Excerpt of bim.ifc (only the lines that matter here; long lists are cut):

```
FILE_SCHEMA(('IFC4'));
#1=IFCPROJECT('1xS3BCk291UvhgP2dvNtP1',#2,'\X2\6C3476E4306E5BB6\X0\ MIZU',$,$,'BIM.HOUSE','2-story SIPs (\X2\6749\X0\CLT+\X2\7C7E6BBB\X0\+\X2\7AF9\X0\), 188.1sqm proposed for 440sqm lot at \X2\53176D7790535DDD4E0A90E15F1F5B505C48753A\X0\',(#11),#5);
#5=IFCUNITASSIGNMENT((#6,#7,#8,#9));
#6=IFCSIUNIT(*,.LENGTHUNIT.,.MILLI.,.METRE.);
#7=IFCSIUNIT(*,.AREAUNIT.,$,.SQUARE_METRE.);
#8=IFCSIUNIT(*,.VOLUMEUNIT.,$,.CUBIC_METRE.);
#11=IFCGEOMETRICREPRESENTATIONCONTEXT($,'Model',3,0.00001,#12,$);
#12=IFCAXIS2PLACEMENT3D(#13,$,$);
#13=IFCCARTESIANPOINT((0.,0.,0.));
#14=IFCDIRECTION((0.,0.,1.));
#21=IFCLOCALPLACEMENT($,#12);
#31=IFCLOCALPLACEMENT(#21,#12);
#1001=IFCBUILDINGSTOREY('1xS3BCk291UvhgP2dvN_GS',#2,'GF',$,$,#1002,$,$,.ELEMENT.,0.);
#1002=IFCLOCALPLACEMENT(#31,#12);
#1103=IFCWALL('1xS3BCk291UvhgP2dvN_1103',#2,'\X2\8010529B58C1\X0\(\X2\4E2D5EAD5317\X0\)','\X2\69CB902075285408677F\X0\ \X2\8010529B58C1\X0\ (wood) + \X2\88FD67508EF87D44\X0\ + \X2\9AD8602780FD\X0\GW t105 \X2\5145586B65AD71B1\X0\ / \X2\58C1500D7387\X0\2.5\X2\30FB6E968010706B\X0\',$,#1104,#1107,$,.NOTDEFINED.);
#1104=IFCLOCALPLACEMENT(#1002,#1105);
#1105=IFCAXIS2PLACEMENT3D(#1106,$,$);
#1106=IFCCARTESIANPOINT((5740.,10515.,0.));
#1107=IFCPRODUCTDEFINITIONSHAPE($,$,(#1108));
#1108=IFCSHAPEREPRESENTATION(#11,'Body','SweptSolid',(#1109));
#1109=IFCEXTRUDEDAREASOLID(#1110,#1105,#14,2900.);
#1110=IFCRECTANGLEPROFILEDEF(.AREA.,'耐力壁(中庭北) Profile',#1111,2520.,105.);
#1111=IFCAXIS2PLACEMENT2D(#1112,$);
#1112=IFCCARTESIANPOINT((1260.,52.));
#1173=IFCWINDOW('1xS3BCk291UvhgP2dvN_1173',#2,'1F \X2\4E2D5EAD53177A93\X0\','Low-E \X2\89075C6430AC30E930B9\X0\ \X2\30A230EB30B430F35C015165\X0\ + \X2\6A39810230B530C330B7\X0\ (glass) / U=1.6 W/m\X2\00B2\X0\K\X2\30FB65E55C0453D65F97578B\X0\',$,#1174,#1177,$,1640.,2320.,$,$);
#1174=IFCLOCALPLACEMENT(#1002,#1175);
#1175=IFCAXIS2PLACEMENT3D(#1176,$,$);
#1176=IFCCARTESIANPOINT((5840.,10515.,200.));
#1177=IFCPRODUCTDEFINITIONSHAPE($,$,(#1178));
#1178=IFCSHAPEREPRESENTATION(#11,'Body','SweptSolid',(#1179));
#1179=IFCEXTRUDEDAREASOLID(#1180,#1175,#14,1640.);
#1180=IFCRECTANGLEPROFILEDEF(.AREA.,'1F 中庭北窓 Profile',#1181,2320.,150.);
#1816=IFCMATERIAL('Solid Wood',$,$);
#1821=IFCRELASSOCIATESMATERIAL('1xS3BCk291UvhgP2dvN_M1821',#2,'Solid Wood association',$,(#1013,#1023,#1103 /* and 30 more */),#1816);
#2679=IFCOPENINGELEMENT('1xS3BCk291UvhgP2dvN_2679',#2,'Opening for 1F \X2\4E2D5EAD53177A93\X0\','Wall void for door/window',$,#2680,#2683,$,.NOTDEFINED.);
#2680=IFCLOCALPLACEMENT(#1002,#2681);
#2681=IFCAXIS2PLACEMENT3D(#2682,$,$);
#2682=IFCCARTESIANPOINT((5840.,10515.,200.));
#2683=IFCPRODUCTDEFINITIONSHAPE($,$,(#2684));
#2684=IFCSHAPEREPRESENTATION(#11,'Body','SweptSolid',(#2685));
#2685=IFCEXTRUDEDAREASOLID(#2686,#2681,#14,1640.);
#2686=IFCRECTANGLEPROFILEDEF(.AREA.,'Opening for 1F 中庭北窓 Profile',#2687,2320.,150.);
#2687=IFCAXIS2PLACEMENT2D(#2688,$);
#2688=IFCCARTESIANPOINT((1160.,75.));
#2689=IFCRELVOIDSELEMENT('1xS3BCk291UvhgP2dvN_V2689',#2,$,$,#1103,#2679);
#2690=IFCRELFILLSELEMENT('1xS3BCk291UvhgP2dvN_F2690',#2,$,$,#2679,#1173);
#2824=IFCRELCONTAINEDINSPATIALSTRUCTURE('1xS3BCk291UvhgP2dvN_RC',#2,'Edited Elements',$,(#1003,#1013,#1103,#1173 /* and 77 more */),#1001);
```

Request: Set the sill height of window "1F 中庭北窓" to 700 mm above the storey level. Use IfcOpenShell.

```python
import numpy as np
import ifcopenshell
import ifcopenshell.api.geometry
import ifcopenshell.geom
import ifcopenshell.util.element
import ifcopenshell.util.placement
import ifcopenshell.util.shape
import ifcopenshell.util.unit

model = ifcopenshell.open("bim.ifc")
unit_scale = ifcopenshell.util.unit.calculate_unit_scale(model)

window = model.by_guid("1xS3BCk291UvhgP2dvN_1173")
opening = window.FillsVoids[0].RelatingOpeningElement
storey = ifcopenshell.util.element.get_container(window, ifc_class="IfcBuildingStorey")
level = ifcopenshell.util.placement.get_local_placement(storey.ObjectPlacement)[2, 3]

# The opening's origin need not be at the sill, so measure its lowest point.
shape = ifcopenshell.geom.create_shape(ifcopenshell.geom.settings(), opening)
bottom = ifcopenshell.util.shape.get_shape_bottom_elevation(shape, shape.geometry) / unit_scale
dz = level + 0.7 / unit_scale - bottom

shift = np.array([0.0, 0.0, dz])
# The window is not placed relative to its opening, so move both.
for product in (opening, window):
    matrix = ifcopenshell.util.placement.get_local_placement(product.ObjectPlacement)
    matrix[:3, 3] += shift
    ifcopenshell.api.geometry.edit_object_placement(model, product=product, matrix=matrix, is_si=False)

print(f"moved by {dz * unit_scale:+.3f} m")

model.write("bim-out.ifc")
```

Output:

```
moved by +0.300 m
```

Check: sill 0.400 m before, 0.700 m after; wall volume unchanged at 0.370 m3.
